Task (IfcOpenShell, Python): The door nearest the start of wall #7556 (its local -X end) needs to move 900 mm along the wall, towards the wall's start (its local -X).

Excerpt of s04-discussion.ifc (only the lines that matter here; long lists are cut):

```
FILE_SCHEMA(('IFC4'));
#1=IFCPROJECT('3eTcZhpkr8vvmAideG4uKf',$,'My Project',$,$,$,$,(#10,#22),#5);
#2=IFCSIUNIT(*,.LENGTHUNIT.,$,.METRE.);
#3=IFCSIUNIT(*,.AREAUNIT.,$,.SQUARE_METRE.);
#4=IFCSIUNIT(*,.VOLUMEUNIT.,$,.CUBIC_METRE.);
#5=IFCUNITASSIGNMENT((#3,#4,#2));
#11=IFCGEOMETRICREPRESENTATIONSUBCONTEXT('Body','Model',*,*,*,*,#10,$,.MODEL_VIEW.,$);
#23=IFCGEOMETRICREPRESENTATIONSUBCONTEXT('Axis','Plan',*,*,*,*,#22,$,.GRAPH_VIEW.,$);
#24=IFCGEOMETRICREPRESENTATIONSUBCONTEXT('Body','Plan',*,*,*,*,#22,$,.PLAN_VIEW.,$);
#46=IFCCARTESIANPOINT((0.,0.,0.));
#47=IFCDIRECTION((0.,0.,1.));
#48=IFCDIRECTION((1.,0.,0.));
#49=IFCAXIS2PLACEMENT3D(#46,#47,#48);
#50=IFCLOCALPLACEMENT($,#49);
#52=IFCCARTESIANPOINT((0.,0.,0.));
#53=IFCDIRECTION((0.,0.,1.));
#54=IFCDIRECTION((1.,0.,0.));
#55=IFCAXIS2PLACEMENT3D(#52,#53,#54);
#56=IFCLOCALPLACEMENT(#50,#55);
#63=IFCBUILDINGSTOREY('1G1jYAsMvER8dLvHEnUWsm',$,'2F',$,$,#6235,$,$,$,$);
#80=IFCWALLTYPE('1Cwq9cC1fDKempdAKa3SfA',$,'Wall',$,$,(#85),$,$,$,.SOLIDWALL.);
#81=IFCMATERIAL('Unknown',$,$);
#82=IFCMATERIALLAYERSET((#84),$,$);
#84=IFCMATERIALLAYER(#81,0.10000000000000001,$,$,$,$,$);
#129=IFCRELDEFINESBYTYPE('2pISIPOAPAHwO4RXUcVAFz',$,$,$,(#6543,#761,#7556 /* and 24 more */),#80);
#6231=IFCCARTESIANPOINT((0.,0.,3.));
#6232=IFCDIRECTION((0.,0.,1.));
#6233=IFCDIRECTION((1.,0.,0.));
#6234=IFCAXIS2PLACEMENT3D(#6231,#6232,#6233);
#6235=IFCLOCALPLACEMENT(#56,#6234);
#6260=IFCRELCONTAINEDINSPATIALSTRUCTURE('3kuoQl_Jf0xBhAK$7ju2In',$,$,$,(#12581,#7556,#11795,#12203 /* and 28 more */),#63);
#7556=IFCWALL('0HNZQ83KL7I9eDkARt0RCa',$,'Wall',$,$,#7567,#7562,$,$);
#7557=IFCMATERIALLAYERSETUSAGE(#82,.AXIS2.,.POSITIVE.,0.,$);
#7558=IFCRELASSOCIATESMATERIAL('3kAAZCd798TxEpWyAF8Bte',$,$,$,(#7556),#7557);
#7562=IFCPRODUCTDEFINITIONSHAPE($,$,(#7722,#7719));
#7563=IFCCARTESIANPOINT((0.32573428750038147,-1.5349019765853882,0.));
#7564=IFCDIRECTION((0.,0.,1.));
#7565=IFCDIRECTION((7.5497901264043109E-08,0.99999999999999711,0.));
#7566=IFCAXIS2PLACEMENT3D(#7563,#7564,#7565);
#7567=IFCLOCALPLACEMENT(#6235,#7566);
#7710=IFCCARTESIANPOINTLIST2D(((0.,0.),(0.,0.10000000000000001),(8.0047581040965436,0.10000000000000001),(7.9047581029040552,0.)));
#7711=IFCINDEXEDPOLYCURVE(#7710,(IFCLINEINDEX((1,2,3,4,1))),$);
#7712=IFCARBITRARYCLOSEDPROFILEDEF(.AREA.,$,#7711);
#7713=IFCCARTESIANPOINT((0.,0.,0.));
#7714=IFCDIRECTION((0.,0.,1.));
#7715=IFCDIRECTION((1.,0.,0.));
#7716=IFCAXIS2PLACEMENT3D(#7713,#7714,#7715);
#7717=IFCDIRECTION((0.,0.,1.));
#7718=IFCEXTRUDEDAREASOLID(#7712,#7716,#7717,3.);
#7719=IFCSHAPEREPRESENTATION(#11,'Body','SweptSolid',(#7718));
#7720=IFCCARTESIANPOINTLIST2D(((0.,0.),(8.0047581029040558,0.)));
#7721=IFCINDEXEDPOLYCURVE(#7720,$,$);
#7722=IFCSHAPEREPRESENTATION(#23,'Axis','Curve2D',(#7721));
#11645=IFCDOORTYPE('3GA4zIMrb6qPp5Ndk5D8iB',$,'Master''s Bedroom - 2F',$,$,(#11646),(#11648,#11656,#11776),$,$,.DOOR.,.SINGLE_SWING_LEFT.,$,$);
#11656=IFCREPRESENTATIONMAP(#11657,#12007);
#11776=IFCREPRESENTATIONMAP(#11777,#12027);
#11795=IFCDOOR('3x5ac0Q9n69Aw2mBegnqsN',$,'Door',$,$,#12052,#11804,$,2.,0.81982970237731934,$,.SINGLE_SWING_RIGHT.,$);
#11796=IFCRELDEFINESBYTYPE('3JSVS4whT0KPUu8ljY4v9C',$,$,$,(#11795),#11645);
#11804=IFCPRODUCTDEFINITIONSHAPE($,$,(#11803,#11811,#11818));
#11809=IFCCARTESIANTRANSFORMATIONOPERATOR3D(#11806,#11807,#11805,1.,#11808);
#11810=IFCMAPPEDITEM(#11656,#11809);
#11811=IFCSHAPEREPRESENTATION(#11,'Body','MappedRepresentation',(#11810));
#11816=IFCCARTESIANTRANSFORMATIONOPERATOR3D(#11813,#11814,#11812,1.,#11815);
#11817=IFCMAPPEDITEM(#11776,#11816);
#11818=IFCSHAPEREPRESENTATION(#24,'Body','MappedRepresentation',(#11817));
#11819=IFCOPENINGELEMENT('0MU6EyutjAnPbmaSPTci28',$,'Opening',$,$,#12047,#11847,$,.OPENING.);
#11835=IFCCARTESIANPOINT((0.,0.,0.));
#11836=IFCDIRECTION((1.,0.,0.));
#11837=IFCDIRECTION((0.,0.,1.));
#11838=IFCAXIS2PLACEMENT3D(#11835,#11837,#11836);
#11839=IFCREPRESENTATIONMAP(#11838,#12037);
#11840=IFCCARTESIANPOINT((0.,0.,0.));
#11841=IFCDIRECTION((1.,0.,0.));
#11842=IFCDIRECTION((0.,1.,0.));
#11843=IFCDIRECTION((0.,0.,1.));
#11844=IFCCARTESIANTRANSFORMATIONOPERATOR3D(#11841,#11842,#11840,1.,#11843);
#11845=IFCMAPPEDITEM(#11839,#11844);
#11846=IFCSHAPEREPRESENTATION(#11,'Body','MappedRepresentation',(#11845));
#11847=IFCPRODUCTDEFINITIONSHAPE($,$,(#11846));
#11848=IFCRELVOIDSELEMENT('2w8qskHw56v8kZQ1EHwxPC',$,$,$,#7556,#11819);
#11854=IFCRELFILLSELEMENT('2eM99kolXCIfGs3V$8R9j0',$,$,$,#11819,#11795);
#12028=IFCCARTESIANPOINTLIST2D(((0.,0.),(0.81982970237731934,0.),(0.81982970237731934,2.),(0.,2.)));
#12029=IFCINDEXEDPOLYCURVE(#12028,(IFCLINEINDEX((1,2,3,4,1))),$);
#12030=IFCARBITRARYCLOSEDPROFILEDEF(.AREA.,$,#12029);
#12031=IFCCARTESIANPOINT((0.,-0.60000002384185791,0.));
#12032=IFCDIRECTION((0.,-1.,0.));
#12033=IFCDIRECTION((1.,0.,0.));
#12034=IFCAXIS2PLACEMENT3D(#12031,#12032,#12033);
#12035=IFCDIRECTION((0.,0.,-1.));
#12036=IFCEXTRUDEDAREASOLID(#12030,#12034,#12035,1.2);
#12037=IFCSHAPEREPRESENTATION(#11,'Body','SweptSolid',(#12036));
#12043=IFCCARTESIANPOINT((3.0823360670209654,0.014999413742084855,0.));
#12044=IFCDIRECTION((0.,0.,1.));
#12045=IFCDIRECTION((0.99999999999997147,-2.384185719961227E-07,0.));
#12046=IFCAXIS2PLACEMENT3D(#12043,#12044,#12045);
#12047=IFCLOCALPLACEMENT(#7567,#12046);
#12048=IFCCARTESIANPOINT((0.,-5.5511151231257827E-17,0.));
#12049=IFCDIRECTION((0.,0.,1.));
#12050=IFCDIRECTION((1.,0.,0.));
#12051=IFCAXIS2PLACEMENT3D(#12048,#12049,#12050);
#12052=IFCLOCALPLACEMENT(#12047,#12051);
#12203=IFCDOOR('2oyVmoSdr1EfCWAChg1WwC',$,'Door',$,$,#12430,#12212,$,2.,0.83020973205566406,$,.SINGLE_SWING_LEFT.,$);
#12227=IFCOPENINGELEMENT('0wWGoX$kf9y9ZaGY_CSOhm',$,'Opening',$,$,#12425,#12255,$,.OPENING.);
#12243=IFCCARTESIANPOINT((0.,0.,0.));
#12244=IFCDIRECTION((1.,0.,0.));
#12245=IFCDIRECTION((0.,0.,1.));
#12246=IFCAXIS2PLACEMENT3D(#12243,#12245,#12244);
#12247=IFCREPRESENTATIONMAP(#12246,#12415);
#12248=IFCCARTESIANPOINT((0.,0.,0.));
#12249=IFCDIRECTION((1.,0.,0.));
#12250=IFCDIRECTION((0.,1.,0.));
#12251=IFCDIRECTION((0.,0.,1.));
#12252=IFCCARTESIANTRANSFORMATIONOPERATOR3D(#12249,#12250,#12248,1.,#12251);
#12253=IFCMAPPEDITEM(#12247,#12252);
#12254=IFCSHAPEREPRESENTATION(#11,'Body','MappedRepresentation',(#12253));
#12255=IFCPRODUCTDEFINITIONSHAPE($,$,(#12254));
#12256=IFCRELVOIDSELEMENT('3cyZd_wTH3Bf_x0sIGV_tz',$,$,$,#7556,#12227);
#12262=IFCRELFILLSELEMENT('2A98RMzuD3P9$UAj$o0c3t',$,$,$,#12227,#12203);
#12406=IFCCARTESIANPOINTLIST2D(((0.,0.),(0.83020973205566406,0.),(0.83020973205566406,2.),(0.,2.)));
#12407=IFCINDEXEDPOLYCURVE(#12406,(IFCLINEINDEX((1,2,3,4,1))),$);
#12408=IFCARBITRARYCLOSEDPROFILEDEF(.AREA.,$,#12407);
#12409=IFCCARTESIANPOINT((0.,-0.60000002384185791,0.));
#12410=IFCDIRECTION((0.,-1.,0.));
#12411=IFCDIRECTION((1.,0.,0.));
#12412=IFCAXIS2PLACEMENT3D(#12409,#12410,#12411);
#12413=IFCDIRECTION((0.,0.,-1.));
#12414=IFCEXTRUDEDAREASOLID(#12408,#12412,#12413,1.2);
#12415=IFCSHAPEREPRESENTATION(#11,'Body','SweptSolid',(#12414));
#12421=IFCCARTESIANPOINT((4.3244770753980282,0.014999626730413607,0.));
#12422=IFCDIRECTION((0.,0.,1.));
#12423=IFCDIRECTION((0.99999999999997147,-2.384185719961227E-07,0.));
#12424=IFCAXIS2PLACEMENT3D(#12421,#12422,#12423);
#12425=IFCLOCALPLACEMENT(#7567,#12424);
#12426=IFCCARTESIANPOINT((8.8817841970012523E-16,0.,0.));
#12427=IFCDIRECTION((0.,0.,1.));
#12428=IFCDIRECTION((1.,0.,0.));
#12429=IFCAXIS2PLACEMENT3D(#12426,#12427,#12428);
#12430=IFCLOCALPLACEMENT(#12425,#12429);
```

```python
import ifcopenshell
import ifcopenshell.api.geometry
import ifcopenshell.util.placement

model = ifcopenshell.open("s04-discussion.ifc")

door = model.by_guid("3x5ac0Q9n69Aw2mBegnqsN")
opening = door.FillsVoids[0].RelatingOpeningElement
wall = opening.VoidsElements[0].RelatingBuildingElement

wall_matrix = ifcopenshell.util.placement.get_local_placement(wall.ObjectPlacement)
shift = wall_matrix[:3, 0] * -0.9
before = ifcopenshell.util.placement.get_local_placement(door.ObjectPlacement)[:3, 3].copy()

# The door is placed relative to its opening, so it follows when the opening moves.
matrix = ifcopenshell.util.placement.get_local_placement(opening.ObjectPlacement)
matrix[:3, 3] += shift
ifcopenshell.api.geometry.edit_object_placement(
    model, product=opening, matrix=matrix, is_si=False, should_transform_children=True
)

after = ifcopenshell.util.placement.get_local_placement(door.ObjectPlacement)[:3, 3]
print("door moved by", (after - before).round(3) + 0.0)

model.write("s04-discussion_rev.ifc")
```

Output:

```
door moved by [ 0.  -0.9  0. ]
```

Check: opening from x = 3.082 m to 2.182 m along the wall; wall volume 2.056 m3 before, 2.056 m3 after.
